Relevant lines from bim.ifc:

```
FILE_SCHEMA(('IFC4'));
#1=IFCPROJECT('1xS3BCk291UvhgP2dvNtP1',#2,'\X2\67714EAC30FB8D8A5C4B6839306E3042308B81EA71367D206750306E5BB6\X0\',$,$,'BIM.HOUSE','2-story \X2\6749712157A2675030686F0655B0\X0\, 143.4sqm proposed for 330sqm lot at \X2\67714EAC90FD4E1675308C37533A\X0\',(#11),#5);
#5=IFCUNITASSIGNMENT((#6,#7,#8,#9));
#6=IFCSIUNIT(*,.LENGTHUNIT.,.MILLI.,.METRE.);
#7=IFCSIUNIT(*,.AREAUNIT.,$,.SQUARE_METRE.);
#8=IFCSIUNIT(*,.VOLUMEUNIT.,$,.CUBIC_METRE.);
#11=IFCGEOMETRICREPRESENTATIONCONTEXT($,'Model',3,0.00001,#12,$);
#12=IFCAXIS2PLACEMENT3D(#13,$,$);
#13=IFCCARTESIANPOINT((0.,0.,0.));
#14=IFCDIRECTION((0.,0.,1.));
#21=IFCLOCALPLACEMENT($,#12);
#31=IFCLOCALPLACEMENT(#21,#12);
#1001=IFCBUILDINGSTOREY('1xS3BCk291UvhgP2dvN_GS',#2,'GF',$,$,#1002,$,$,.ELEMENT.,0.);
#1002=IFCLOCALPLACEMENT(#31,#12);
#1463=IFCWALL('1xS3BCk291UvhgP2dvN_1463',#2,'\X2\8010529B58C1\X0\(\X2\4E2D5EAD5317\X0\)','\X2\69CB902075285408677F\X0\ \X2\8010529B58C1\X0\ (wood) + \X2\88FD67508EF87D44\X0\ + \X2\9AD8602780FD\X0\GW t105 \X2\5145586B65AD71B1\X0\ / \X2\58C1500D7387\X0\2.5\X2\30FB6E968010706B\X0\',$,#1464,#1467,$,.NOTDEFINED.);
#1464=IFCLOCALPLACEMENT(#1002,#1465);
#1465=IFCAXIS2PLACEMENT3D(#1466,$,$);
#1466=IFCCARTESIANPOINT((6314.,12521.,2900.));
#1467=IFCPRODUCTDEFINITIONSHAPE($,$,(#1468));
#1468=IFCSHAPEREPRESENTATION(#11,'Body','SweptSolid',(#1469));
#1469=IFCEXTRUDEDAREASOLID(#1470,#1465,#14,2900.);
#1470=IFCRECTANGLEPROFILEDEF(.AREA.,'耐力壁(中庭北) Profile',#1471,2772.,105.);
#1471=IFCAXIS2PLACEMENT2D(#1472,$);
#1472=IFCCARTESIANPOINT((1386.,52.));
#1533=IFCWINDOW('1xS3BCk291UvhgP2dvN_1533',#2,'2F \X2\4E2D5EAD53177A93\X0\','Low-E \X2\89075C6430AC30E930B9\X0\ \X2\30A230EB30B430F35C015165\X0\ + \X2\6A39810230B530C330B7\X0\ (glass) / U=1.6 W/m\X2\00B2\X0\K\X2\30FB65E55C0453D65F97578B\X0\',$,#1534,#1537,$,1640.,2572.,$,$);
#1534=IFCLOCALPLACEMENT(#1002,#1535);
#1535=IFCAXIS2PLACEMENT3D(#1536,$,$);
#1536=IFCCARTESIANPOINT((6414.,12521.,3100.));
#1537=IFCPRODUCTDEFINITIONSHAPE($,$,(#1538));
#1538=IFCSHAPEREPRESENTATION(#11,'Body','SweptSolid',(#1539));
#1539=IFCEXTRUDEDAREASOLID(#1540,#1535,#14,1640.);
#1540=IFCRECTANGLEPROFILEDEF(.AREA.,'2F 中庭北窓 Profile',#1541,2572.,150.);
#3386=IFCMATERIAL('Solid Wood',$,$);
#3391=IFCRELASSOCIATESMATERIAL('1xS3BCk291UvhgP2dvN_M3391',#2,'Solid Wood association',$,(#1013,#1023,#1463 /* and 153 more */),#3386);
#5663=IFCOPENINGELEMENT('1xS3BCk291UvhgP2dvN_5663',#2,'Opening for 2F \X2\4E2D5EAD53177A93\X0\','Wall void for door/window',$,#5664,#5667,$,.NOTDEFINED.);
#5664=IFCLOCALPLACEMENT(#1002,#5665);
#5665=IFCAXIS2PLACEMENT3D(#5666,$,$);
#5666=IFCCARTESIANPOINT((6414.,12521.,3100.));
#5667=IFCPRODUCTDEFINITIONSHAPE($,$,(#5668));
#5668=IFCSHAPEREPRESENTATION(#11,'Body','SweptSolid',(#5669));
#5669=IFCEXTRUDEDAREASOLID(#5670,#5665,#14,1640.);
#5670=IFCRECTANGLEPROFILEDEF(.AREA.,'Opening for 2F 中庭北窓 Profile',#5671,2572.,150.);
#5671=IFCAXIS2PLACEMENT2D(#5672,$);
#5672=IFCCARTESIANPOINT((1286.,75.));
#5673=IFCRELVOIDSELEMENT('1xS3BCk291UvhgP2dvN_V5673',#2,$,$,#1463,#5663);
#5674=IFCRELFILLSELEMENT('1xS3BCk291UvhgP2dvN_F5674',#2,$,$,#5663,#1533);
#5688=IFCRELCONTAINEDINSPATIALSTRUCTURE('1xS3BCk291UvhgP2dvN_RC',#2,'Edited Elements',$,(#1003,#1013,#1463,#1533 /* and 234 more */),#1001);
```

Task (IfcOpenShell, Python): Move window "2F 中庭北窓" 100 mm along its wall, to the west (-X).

```python
import ifcopenshell
import ifcopenshell.api.geometry
import ifcopenshell.util.placement
import ifcopenshell.util.unit

model = ifcopenshell.open("bim.ifc")
unit_scale = ifcopenshell.util.unit.calculate_unit_scale(model)

window = model.by_guid("1xS3BCk291UvhgP2dvN_1533")
opening = window.FillsVoids[0].RelatingOpeningElement
wall = opening.VoidsElements[0].RelatingBuildingElement

wall_matrix = ifcopenshell.util.placement.get_local_placement(wall.ObjectPlacement)
shift = wall_matrix[:3, 0] * -0.1 / unit_scale
before = ifcopenshell.util.placement.get_local_placement(window.ObjectPlacement)[:3, 3].copy()

# The window is not placed relative to its opening, so move both.
for product in (opening, window):
    matrix = ifcopenshell.util.placement.get_local_placement(product.ObjectPlacement)
    matrix[:3, 3] += shift
    ifcopenshell.api.geometry.edit_object_placement(model, product=product, matrix=matrix, is_si=False)

after = ifcopenshell.util.placement.get_local_placement(window.ObjectPlacement)[:3, 3]
print("window moved by", (after - before).round(3) + 0.0)

model.write("bim_edited.ifc")
```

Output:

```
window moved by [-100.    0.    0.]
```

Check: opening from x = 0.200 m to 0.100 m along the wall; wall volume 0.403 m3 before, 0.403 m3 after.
